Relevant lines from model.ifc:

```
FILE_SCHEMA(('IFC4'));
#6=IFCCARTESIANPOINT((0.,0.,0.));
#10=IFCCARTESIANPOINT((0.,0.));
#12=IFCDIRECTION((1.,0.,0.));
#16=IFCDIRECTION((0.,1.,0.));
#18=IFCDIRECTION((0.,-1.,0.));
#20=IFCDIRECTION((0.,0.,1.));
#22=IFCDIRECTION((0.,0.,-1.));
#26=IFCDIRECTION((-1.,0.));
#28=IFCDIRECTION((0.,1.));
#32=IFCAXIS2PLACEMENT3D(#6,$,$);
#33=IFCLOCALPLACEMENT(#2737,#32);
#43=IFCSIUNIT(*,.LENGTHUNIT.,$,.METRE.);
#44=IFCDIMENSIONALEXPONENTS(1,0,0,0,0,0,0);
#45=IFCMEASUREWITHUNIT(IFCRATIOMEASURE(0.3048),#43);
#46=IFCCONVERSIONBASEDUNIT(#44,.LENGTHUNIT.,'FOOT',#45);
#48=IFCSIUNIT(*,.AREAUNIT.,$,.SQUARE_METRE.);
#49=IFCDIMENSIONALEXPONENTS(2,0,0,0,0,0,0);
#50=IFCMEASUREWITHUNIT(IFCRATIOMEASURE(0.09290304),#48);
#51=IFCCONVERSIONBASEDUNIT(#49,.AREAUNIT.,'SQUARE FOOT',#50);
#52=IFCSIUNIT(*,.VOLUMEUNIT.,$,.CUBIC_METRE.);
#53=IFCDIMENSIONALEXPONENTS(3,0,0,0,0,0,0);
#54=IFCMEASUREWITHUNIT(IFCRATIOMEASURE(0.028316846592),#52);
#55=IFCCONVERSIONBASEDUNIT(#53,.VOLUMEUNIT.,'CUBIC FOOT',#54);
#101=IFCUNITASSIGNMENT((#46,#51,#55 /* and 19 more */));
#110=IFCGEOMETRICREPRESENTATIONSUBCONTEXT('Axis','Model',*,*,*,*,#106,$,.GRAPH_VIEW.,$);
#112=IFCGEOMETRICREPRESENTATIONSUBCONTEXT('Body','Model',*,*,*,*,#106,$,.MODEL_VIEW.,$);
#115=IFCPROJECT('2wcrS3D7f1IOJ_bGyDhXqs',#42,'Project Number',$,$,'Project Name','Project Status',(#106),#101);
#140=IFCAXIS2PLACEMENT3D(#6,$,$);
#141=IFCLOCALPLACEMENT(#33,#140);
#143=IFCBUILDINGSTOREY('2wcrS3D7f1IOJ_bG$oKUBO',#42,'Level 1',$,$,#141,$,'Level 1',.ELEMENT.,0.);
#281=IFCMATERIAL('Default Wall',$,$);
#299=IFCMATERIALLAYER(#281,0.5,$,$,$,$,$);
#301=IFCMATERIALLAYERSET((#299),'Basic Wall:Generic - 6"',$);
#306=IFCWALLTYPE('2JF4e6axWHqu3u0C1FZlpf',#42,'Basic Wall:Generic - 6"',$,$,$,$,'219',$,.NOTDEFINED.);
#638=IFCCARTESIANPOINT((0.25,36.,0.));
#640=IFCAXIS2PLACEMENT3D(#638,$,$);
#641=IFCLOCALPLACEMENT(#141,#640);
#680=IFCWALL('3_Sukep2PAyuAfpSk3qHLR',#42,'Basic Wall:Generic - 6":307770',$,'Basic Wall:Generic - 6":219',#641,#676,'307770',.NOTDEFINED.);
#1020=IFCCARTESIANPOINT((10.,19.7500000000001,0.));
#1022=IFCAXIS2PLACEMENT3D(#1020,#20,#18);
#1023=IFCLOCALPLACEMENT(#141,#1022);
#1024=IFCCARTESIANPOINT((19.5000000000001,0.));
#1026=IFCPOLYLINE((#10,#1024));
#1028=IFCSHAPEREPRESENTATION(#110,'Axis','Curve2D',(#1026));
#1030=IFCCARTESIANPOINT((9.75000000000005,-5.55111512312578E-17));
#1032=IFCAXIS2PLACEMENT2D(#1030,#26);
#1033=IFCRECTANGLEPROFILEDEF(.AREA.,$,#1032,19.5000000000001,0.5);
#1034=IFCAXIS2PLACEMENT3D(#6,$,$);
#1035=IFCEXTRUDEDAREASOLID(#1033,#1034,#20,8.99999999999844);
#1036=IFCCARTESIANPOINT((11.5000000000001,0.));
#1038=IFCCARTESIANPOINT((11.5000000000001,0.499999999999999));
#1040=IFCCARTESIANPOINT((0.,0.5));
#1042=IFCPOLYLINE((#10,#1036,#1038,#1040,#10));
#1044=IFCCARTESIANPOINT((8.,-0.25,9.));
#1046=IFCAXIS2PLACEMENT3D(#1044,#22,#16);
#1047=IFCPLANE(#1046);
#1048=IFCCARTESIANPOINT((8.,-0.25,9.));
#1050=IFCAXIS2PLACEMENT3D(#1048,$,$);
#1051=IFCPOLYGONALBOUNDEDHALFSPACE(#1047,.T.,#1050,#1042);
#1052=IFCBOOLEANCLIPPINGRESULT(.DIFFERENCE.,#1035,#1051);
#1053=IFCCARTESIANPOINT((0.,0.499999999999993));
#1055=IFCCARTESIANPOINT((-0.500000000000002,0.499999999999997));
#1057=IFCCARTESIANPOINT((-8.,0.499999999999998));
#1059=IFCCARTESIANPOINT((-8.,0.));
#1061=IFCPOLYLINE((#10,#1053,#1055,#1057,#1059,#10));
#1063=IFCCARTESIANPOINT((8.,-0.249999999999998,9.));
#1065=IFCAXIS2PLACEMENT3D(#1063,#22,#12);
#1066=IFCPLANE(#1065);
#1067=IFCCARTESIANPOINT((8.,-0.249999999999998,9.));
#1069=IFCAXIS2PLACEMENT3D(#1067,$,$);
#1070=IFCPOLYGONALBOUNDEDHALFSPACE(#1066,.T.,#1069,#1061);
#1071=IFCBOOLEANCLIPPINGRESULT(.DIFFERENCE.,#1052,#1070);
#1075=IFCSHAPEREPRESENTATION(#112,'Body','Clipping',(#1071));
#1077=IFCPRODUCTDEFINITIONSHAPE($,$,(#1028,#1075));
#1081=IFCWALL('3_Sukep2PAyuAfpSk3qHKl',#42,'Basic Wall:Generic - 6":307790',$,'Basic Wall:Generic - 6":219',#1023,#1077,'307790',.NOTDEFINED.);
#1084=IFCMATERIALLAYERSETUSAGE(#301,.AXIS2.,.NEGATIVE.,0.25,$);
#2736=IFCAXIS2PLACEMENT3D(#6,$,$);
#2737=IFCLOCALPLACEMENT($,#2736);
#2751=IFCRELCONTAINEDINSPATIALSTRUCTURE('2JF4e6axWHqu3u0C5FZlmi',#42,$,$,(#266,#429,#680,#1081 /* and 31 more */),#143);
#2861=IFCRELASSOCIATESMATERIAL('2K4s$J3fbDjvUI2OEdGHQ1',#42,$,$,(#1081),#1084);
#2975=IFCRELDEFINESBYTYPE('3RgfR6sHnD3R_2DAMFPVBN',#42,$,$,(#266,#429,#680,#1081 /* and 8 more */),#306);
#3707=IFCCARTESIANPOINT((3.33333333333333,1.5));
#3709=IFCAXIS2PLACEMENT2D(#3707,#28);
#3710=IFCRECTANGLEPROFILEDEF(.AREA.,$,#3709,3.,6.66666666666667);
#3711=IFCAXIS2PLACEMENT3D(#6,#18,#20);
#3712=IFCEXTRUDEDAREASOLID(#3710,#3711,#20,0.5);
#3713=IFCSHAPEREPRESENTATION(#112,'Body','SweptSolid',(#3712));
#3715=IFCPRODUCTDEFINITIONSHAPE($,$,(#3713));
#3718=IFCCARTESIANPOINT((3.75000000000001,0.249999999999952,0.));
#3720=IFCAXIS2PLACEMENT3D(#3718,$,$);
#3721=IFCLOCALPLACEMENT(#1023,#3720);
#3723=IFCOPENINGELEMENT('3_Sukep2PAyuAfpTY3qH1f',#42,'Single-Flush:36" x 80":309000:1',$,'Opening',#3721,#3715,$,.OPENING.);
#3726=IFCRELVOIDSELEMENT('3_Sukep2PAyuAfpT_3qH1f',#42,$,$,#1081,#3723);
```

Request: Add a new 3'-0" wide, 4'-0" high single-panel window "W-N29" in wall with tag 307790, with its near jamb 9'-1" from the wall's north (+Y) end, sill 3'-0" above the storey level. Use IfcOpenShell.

```python
import numpy as np
import ifcopenshell
import ifcopenshell.api.feature
import ifcopenshell.api.geometry
import ifcopenshell.api.root
import ifcopenshell.api.spatial
import ifcopenshell.geom
import ifcopenshell.util.element
import ifcopenshell.util.placement
import ifcopenshell.util.representation
import ifcopenshell.util.shape
import ifcopenshell.util.unit

model = ifcopenshell.open("model.ifc")
unit_scale = ifcopenshell.util.unit.calculate_unit_scale(model)
settings = ifcopenshell.geom.settings()


def volume(element):
    """Net volume in cubic metres, openings subtracted."""
    shape = ifcopenshell.geom.create_shape(settings, element)
    return ifcopenshell.util.shape.get_volume(shape.geometry)


wall = model.by_guid("3_Sukep2PAyuAfpSk3qHKl")
storey = ifcopenshell.util.element.get_container(wall, ifc_class="IfcBuildingStorey")
context = ifcopenshell.util.representation.get_context(model, "Model", "Body", "MODEL_VIEW")
before = volume(wall)

width, height, from_end, sill = 0.9144, 1.2192, 2.7686, 0.9144  # metres

# The wall runs along its own X axis, and the end named is its -X end.
wall_shape = ifcopenshell.geom.create_shape(settings, wall)
x, y, z = ifcopenshell.util.shape.get_vertices(wall_shape.geometry).T
start = x.min() + from_end
face, thickness = float(y.min()), float(y.max() - y.min())
wall_matrix = ifcopenshell.util.placement.get_local_placement(wall.ObjectPlacement)
level = ifcopenshell.util.placement.get_local_placement(storey.ObjectPlacement)[2, 3]


def in_wall(x, y):
    """Placement at x, y metres in the wall's axes, at sill height."""
    matrix = wall_matrix.copy()
    matrix[:, 3] = wall_matrix @ np.array([x / unit_scale, y / unit_scale, 0.0, 1.0])
    matrix[2, 3] = level + sill / unit_scale
    return matrix


# Opening: a box that overshoots both wall faces by 50 mm.
opening = ifcopenshell.api.root.create_entity(model, ifc_class="IfcOpeningElement", predefined_type="OPENING")
box = ifcopenshell.api.geometry.add_wall_representation(
    model, context=context, length=width, height=height, thickness=thickness + 0.1
)
ifcopenshell.api.geometry.assign_representation(model, product=opening, representation=box)
ifcopenshell.api.geometry.edit_object_placement(model, product=opening, matrix=in_wall(start, face - 0.05), is_si=False)
ifcopenshell.api.feature.add_feature(model, feature=opening, element=wall)

window = ifcopenshell.api.root.create_entity(model, ifc_class="IfcWindow", name="W-N29", predefined_type="WINDOW")
window.OverallWidth, window.OverallHeight = width / unit_scale, height / unit_scale
window.PartitioningType = "SINGLE_PANEL"
body = ifcopenshell.api.geometry.add_window_representation(
    model,
    context=context,
    overall_width=window.OverallWidth,
    overall_height=window.OverallHeight,
    partition_type="SINGLE_PANEL",
)
ifcopenshell.api.geometry.assign_representation(model, product=window, representation=body)
ifcopenshell.api.spatial.assign_container(model, products=[window], relating_structure=storey)
ifcopenshell.api.feature.add_filling(model, opening=opening, element=window)

# Centre the window in the wall's thickness.
ifcopenshell.api.geometry.edit_object_placement(model, product=window, matrix=in_wall(start, face), is_si=False)
window_shape = ifcopenshell.geom.create_shape(settings, window)
depth = ifcopenshell.util.shape.get_vertices(window_shape.geometry)[:, 1]
offset = face + thickness / 2 - (depth.min() + depth.max()) / 2
ifcopenshell.api.geometry.edit_object_placement(model, product=window, matrix=in_wall(start, offset), is_si=False)

after = volume(wall)

print(f"wall volume {before:.3f} -> {after:.3f} m3")

model.write("model_rev.ifc")
```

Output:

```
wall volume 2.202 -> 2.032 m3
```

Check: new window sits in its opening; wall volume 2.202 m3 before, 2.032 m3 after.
